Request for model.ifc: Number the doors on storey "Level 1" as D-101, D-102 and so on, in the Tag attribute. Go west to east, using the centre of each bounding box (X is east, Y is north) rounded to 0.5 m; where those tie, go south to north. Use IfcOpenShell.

First a look at what the model holds.

```python
import ifcopenshell
import ifcopenshell.util.element
import ifcopenshell.util.placement

model = ifcopenshell.open("model.ifc")
print(model.schema)
storey = next(s for s in model.by_type("IfcBuildingStorey") if s.Name == "Level 1")
doors = [e for e in ifcopenshell.util.element.get_decomposition(storey) if e.is_a("IfcDoor")]
for e in sorted(doors, key=lambda e: e.id()):
    origin = ifcopenshell.util.placement.get_local_placement(e.ObjectPlacement)[:3, 3]
    print(e.id(), e.Tag, e.Name, origin.round(2) + 0.0, sep=" | ")
```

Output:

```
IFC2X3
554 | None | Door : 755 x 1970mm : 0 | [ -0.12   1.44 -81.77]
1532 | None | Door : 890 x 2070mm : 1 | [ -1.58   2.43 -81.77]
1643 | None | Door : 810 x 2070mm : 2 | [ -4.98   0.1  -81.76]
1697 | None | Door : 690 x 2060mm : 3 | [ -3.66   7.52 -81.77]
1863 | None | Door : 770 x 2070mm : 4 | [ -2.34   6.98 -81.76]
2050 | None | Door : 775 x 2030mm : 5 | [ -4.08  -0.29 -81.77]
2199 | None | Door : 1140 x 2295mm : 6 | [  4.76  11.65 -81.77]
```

```python
import ifcopenshell
import ifcopenshell.geom
import ifcopenshell.util.element
import ifcopenshell.util.shape

model = ifcopenshell.open("model.ifc")
settings = ifcopenshell.geom.settings()
settings.set("use-world-coords", True)


def centre(element):
    shape = ifcopenshell.geom.create_shape(settings, element)
    return ifcopenshell.util.shape.get_bbox_centroid(shape.geometry)


storey = next(s for s in model.by_type("IfcBuildingStorey") if s.Name == "Level 1")
doors = [e for e in ifcopenshell.util.element.get_decomposition(storey) if e.is_a("IfcDoor")]

# Insertion points can sit at a corner or the storey origin, so sort by the geometry (in metres).
centres = {e: centre(e) for e in doors}
doors.sort(key=lambda e: (round(centres[e][0] / 0.5), centres[e][1]))

for i, e in enumerate(doors, start=1):
    number = f"D-1{i:02d}"
    e.Tag = number
    print(e.id(), number)

model.write("model_updated.ifc")
```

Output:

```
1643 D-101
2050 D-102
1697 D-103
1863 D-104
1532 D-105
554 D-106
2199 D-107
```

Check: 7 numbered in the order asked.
